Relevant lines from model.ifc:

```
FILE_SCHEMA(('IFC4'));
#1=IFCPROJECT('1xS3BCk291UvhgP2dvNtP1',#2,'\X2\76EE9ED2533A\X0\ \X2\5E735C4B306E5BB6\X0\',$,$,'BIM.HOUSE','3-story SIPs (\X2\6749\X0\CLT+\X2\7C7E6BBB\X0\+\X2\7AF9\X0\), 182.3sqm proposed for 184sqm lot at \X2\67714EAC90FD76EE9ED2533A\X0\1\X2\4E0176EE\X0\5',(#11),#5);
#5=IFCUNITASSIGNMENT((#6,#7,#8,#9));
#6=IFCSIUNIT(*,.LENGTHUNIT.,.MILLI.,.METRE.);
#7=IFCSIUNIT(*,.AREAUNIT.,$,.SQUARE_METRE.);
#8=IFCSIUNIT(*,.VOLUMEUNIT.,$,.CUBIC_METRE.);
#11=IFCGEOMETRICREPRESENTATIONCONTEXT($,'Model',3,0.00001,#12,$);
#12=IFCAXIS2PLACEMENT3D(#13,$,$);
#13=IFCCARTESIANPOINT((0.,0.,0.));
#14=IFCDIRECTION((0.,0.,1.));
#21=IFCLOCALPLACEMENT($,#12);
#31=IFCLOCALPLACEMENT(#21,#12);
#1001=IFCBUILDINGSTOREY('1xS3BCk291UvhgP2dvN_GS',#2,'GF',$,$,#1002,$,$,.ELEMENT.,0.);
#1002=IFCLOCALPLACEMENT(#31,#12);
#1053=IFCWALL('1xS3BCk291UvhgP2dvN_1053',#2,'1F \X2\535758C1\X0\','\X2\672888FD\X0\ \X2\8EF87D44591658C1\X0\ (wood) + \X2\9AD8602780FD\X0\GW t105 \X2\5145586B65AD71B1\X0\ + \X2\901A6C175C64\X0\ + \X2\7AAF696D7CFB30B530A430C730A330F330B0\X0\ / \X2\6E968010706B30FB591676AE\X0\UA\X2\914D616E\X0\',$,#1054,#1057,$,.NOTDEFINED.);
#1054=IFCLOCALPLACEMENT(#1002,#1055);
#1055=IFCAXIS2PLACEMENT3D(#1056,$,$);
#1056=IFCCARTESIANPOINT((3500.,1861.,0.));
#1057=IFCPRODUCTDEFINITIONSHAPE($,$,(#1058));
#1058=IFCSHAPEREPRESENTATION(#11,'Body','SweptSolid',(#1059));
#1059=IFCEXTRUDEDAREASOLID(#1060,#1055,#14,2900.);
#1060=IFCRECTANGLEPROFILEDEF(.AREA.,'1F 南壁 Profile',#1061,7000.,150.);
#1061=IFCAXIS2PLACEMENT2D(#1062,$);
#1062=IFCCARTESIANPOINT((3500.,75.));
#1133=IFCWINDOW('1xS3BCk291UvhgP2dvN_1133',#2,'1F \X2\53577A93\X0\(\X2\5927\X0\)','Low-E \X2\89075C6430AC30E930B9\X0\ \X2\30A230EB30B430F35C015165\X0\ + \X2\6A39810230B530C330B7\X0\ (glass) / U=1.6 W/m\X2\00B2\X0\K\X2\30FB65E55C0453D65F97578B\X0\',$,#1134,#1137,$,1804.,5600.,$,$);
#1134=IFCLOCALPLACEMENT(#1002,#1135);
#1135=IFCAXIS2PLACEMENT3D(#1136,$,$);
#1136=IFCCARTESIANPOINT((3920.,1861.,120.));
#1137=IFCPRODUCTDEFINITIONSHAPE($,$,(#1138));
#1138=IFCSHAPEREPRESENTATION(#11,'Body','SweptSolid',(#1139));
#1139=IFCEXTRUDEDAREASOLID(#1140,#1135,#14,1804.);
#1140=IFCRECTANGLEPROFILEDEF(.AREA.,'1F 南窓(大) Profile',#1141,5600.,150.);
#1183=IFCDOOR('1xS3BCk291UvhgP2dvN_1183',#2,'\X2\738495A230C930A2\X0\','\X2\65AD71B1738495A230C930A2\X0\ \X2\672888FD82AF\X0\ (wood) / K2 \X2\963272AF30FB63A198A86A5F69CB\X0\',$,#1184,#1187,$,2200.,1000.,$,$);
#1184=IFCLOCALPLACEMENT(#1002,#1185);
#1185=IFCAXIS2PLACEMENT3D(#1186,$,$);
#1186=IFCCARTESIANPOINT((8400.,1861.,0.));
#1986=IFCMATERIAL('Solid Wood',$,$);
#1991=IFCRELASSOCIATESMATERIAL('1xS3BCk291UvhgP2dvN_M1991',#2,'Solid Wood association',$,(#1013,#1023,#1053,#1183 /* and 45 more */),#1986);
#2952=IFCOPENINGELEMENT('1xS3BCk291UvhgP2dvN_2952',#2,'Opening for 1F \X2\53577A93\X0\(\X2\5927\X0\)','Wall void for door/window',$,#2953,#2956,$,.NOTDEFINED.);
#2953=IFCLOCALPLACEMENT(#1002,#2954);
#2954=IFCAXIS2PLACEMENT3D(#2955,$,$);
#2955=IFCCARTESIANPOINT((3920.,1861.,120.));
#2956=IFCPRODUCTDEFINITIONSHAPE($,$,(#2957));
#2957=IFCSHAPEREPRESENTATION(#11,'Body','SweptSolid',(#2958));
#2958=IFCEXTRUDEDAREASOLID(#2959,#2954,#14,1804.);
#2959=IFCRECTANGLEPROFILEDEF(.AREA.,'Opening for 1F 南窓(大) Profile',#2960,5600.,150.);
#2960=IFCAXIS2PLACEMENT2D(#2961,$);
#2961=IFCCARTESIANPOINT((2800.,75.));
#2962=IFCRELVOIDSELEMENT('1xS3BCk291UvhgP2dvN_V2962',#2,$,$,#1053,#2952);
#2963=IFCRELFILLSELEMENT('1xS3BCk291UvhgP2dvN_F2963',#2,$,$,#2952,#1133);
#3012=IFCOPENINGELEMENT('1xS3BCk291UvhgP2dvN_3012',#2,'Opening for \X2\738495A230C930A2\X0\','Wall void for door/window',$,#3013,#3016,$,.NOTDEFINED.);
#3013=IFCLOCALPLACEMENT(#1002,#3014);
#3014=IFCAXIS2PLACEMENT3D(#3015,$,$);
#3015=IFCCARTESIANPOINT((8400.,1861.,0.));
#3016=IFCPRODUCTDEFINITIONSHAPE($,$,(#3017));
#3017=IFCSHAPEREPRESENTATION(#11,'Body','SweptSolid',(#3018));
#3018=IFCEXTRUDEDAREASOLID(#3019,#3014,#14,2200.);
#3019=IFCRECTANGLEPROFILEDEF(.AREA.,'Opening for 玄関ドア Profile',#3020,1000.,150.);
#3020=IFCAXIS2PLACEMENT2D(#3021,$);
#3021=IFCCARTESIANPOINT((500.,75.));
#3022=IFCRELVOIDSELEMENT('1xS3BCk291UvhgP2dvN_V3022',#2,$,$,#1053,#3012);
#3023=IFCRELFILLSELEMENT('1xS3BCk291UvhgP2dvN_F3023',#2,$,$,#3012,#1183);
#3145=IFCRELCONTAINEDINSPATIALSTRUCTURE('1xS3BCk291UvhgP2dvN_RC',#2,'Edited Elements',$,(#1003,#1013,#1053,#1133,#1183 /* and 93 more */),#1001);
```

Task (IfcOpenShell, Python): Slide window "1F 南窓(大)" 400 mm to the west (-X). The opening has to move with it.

```python
import ifcopenshell
import ifcopenshell.api.geometry
import ifcopenshell.util.placement
import ifcopenshell.util.unit

model = ifcopenshell.open("model.ifc")
unit_scale = ifcopenshell.util.unit.calculate_unit_scale(model)

window = model.by_guid("1xS3BCk291UvhgP2dvN_1133")
opening = window.FillsVoids[0].RelatingOpeningElement
wall = opening.VoidsElements[0].RelatingBuildingElement

wall_matrix = ifcopenshell.util.placement.get_local_placement(wall.ObjectPlacement)
shift = wall_matrix[:3, 0] * -0.4 / unit_scale
before = ifcopenshell.util.placement.get_local_placement(window.ObjectPlacement)[:3, 3].copy()

# The window is not placed relative to its opening, so move both.
for product in (opening, window):
    matrix = ifcopenshell.util.placement.get_local_placement(product.ObjectPlacement)
    matrix[:3, 3] += shift
    ifcopenshell.api.geometry.edit_object_placement(model, product=product, matrix=matrix, is_si=False)

after = ifcopenshell.util.placement.get_local_placement(window.ObjectPlacement)[:3, 3]
print("window moved by", (after - before).round(3) + 0.0)

model.write("model-out.ifc")
```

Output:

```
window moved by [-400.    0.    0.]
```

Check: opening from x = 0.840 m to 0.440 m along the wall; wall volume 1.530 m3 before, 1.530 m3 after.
